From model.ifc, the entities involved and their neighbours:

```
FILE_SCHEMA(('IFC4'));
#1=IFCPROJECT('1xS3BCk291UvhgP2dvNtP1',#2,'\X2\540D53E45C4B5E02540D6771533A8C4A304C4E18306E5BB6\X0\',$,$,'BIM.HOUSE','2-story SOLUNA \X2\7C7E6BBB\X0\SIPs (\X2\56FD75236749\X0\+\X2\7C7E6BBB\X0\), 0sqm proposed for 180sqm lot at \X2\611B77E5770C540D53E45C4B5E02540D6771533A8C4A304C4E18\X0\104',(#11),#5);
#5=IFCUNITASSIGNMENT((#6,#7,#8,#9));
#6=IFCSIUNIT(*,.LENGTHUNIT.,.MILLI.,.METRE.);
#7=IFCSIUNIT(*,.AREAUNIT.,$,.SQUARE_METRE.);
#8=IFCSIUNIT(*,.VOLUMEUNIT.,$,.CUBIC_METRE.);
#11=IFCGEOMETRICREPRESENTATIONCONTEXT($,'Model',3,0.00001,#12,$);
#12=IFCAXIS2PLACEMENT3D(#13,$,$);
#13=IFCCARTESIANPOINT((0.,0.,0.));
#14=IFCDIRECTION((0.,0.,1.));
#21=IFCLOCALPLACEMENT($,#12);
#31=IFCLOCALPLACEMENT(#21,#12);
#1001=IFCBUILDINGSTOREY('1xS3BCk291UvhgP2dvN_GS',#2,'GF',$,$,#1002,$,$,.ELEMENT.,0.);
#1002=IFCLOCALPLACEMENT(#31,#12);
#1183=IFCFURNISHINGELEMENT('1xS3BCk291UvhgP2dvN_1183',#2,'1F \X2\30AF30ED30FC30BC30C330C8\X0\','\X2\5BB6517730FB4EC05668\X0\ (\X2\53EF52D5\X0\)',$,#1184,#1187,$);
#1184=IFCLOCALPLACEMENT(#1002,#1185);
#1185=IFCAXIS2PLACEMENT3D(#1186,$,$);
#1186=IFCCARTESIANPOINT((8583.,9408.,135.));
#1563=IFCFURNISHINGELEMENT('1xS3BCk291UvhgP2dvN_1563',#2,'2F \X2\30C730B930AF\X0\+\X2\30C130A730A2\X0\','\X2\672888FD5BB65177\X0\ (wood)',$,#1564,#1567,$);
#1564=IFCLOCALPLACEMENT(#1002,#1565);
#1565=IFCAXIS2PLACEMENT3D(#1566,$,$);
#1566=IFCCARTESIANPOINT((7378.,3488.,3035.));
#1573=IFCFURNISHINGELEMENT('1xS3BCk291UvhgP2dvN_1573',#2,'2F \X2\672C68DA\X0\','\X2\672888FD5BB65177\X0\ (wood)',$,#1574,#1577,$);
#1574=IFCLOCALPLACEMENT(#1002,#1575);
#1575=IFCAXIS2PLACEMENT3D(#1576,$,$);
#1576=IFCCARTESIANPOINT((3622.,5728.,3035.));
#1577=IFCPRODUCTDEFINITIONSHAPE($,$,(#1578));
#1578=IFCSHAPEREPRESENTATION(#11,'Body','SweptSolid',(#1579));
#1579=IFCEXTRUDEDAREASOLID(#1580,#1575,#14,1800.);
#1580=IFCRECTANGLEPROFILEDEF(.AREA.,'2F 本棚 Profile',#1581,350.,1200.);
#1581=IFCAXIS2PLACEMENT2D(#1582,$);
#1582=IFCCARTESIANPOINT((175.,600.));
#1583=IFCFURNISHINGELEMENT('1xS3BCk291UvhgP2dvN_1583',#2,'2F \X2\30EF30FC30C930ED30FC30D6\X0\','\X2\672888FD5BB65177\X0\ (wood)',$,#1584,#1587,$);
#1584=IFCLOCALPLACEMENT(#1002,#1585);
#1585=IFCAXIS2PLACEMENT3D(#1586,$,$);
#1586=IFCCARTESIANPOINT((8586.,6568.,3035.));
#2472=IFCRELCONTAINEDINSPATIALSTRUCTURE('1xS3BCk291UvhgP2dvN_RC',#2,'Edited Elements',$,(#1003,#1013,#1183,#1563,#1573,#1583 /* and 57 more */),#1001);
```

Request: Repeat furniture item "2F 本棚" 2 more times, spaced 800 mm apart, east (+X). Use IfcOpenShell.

```python
import numpy as np
import ifcopenshell
import ifcopenshell.api.geometry
import ifcopenshell.api.root
import ifcopenshell.util.element
import ifcopenshell.util.placement

model = ifcopenshell.open("model.ifc")


def reuse_history(source, copy):
    """copy_class also copies each property set's owner history, people and application; keep the originals."""
    for rel in copy.IsDefinedBy:
        if rel.is_a("IfcRelDefinesByProperties") and (history := rel.RelatingPropertyDefinition.OwnerHistory):
            rel.RelatingPropertyDefinition.OwnerHistory = source.OwnerHistory
            ifcopenshell.util.element.remove_deep2(model, history)


source = model.by_guid("1xS3BCk291UvhgP2dvN_1573")
base = ifcopenshell.util.placement.get_local_placement(source.ObjectPlacement)
step = np.array([1.0, 0.0, 0.0]) * 800.0

for i in range(1, 3):
    copy = ifcopenshell.api.root.copy_class(model, product=source)
    copy.Representation = ifcopenshell.util.element.copy_deep(
        model, source.Representation, exclude=["IfcGeometricRepresentationContext", "IfcRepresentationMap"]
    )
    reuse_history(source, copy)
    matrix = base.copy()
    matrix[:3, 3] += i * step
    print("added at", matrix[:3, 3].round(3) + 0.0)
    ifcopenshell.api.geometry.edit_object_placement(model, product=copy, matrix=matrix, is_si=False)

model.write("model_updated.ifc")
```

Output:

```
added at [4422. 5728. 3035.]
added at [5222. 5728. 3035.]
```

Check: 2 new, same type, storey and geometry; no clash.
